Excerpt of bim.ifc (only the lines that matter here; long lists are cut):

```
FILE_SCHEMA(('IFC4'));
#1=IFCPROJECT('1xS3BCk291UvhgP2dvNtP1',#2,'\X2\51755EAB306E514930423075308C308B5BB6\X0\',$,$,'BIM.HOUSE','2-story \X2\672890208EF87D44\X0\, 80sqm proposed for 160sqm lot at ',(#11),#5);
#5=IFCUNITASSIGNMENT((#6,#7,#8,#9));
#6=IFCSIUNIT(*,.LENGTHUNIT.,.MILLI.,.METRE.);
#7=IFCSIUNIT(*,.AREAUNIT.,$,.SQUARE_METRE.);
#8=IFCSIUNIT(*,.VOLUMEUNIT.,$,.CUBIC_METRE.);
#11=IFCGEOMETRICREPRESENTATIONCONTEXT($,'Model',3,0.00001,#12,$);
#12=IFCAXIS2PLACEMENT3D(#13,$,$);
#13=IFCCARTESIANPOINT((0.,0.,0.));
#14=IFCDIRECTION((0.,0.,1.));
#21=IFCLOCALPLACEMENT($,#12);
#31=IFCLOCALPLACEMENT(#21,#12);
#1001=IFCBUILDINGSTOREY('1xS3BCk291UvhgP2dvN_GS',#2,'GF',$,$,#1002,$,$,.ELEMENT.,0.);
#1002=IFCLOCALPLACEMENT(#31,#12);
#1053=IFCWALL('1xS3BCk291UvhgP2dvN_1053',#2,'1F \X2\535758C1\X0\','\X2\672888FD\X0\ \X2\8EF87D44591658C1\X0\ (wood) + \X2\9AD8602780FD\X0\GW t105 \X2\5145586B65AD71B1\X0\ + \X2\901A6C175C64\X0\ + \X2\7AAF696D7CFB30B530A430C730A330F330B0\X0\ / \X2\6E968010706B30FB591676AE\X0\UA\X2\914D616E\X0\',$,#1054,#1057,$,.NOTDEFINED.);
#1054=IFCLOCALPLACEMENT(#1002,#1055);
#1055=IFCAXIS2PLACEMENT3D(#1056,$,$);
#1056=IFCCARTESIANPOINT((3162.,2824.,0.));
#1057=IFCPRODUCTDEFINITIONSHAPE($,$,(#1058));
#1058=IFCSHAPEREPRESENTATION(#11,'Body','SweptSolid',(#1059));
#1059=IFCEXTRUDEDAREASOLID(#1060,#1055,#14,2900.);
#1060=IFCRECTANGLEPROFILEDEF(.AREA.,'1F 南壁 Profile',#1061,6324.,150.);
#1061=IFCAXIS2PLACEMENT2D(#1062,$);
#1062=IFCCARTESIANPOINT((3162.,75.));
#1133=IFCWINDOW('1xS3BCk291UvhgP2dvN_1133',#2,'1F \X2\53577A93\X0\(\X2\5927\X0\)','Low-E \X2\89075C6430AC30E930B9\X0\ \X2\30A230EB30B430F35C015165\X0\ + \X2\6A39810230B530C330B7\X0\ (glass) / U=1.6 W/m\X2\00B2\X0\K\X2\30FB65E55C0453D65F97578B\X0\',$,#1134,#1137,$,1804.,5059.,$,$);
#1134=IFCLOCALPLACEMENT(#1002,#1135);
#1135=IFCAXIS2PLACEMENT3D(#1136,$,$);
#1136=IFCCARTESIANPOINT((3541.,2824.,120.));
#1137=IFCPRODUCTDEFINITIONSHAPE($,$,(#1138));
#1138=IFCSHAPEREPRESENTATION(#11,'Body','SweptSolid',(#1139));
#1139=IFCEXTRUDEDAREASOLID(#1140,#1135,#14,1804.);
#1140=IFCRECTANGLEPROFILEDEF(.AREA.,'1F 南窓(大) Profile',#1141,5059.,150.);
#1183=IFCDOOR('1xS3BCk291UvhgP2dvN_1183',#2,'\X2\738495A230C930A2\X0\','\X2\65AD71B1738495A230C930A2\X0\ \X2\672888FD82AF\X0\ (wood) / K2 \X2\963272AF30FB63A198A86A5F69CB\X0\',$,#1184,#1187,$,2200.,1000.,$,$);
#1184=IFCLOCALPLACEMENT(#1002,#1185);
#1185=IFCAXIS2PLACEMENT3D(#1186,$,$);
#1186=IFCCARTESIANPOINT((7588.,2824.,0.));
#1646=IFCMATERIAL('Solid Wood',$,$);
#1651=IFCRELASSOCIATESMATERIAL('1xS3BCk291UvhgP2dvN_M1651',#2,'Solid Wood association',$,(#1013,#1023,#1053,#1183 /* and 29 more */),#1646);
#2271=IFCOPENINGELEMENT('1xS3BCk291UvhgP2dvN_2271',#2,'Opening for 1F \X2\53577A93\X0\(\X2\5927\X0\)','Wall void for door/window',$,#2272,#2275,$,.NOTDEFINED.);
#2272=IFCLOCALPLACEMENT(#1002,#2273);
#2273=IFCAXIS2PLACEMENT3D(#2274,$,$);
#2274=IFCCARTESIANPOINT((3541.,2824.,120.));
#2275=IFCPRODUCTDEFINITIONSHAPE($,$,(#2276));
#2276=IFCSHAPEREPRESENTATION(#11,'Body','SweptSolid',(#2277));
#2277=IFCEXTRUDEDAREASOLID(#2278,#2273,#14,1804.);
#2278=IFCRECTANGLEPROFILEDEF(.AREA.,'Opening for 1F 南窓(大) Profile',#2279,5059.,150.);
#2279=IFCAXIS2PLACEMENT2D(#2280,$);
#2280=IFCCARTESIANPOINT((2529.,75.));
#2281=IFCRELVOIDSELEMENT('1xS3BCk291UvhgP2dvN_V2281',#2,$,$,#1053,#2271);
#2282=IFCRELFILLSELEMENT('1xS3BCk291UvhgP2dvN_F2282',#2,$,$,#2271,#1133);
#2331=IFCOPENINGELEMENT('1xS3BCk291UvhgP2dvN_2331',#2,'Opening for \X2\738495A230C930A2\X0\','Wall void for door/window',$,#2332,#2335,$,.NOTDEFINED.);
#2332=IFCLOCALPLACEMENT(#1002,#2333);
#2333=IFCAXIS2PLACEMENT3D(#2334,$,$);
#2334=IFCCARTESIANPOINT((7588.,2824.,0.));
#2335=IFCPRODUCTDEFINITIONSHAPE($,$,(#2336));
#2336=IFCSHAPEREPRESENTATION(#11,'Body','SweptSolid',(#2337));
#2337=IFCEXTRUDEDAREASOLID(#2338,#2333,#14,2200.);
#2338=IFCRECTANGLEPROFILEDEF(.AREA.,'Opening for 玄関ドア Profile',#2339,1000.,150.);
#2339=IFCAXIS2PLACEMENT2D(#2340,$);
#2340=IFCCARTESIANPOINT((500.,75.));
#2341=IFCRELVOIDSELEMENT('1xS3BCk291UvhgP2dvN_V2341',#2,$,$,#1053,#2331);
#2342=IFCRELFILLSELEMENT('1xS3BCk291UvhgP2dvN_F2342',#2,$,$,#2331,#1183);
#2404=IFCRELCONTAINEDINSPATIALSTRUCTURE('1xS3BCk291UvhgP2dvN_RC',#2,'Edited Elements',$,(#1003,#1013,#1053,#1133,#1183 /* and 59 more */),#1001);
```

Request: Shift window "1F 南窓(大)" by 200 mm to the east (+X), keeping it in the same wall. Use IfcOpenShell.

```python
import ifcopenshell
import ifcopenshell.api.geometry
import ifcopenshell.util.placement

model = ifcopenshell.open("bim.ifc")

window = model.by_guid("1xS3BCk291UvhgP2dvN_1133")
opening = window.FillsVoids[0].RelatingOpeningElement
wall = opening.VoidsElements[0].RelatingBuildingElement

wall_matrix = ifcopenshell.util.placement.get_local_placement(wall.ObjectPlacement)
shift = wall_matrix[:3, 0] * 200.0
before = ifcopenshell.util.placement.get_local_placement(window.ObjectPlacement)[:3, 3].copy()

# The window is not placed relative to its opening, so move both.
for product in (opening, window):
    matrix = ifcopenshell.util.placement.get_local_placement(product.ObjectPlacement)
    matrix[:3, 3] += shift
    ifcopenshell.api.geometry.edit_object_placement(model, product=product, matrix=matrix, is_si=False)

after = ifcopenshell.util.placement.get_local_placement(window.ObjectPlacement)[:3, 3]
print("window moved by", (after - before).round(3) + 0.0)

model.write("bim_v2.ifc")
```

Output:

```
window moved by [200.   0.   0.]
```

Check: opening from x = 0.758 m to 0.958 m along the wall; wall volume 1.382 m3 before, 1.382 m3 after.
